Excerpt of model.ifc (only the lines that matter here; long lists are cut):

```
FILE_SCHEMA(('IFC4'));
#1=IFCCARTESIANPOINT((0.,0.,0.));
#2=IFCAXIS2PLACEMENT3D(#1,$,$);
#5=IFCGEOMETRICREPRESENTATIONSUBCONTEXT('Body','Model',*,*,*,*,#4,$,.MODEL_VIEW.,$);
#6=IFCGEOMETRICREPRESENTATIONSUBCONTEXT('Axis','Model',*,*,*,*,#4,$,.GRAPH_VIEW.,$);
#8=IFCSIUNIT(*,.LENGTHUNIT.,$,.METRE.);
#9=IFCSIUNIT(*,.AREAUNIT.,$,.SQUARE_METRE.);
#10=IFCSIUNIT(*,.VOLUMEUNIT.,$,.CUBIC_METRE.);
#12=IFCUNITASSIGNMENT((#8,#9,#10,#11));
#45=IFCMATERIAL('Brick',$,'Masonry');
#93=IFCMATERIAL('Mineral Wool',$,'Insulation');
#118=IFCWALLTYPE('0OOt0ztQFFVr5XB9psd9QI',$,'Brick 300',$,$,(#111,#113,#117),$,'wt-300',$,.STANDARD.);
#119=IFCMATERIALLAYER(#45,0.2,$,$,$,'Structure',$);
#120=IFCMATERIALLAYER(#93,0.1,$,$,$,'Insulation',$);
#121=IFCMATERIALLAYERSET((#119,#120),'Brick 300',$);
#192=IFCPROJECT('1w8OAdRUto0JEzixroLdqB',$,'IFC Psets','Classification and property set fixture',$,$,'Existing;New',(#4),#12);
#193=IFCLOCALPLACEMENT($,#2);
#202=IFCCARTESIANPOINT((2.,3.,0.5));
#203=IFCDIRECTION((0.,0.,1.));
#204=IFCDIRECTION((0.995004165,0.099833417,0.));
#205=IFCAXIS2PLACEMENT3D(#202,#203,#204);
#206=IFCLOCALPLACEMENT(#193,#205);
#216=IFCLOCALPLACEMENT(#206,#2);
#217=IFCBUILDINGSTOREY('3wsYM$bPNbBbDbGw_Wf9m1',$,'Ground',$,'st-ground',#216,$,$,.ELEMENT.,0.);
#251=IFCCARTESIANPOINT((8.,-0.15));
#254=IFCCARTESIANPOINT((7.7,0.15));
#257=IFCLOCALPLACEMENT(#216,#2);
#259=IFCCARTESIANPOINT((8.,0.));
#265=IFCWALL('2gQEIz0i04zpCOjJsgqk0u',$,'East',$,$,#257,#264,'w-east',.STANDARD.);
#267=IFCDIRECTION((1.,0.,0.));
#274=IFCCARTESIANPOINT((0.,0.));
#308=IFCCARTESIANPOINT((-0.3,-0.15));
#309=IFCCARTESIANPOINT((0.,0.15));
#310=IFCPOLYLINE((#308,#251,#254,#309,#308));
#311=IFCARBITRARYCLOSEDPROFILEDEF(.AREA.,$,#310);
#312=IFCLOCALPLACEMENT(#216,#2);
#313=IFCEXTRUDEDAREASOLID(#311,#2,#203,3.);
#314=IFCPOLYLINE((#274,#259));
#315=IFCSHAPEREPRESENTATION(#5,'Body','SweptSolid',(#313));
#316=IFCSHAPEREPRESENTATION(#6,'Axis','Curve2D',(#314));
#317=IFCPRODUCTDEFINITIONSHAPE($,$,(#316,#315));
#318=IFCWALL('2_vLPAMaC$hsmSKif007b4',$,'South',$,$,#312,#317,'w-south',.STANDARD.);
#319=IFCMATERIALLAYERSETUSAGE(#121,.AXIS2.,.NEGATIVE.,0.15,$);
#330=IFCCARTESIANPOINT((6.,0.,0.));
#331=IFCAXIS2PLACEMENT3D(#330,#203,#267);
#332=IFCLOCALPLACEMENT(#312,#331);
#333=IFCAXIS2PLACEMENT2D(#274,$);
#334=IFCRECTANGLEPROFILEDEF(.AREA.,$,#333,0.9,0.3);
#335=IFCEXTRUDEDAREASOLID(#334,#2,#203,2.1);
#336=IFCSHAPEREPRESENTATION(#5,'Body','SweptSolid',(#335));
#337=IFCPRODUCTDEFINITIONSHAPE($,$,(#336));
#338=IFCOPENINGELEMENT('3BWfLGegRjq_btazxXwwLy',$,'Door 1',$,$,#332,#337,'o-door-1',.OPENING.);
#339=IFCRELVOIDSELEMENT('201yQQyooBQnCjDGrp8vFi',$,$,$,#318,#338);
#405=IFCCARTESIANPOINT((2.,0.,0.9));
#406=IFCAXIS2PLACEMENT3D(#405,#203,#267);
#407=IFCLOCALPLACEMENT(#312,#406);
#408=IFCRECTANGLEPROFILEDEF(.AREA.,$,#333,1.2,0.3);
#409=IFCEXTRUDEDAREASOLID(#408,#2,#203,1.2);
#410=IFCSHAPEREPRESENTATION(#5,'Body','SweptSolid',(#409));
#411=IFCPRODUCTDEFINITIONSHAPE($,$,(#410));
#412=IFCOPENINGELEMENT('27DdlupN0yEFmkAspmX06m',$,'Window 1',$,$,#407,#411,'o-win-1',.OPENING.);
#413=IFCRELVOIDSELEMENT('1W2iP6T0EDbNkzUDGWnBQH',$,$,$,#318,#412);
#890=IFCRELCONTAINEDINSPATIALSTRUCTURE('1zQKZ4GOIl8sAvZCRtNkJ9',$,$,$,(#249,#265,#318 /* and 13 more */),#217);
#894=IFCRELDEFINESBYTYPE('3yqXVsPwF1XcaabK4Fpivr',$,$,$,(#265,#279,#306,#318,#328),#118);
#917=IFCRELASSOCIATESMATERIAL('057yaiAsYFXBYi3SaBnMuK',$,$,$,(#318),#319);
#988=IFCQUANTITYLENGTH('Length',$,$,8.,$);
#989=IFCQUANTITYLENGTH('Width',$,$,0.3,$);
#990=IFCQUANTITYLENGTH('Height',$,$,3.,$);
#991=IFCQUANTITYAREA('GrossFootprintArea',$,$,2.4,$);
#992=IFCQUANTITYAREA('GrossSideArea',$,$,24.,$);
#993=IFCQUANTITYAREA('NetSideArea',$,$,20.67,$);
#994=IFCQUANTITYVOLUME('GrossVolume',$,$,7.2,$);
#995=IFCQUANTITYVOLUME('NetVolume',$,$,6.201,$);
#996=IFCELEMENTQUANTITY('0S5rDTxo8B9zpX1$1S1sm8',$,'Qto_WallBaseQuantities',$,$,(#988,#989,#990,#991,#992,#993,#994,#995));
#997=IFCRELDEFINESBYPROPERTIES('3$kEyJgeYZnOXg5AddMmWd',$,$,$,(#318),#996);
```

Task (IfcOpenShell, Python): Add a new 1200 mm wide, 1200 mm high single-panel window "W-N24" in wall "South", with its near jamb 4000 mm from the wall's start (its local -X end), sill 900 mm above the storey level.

```python
import numpy as np
import ifcopenshell
import ifcopenshell.api.feature
import ifcopenshell.api.geometry
import ifcopenshell.api.pset
import ifcopenshell.api.root
import ifcopenshell.api.spatial
import ifcopenshell.geom
import ifcopenshell.util.element
import ifcopenshell.util.placement
import ifcopenshell.util.representation
import ifcopenshell.util.shape
import ifcopenshell.util.unit

model = ifcopenshell.open("model.ifc")
unit_scale = ifcopenshell.util.unit.calculate_unit_scale(model)
area_scale = ifcopenshell.util.unit.calculate_unit_scale(model, "AREAUNIT")
volume_scale = ifcopenshell.util.unit.calculate_unit_scale(model, "VOLUMEUNIT")
settings = ifcopenshell.geom.settings()


def volume(element):
    """Net volume in cubic metres, openings subtracted."""
    shape = ifcopenshell.geom.create_shape(settings, element)
    return ifcopenshell.util.shape.get_volume(shape.geometry)


wall = model.by_guid("2_vLPAMaC$hsmSKif007b4")
storey = ifcopenshell.util.element.get_container(wall, ifc_class="IfcBuildingStorey")
context = ifcopenshell.util.representation.get_context(model, "Model", "Body", "MODEL_VIEW")
before = volume(wall)

width, height, from_end, sill = 1.2, 1.2, 4, 0.9  # metres

# The wall runs along its own X axis, and the end named is its -X end.
wall_shape = ifcopenshell.geom.create_shape(settings, wall)
x, y, z = ifcopenshell.util.shape.get_vertices(wall_shape.geometry).T
start = x.min() + from_end
face, thickness = float(y.min()), float(y.max() - y.min())
wall_matrix = ifcopenshell.util.placement.get_local_placement(wall.ObjectPlacement)
level = ifcopenshell.util.placement.get_local_placement(storey.ObjectPlacement)[2, 3]


def in_wall(x, y):
    """Placement at x, y metres in the wall's axes, at sill height."""
    matrix = wall_matrix.copy()
    matrix[:, 3] = wall_matrix @ np.array([x / unit_scale, y / unit_scale, 0.0, 1.0])
    matrix[2, 3] = level + sill / unit_scale
    return matrix


# Opening: a box that overshoots both wall faces by 50 mm.
opening = ifcopenshell.api.root.create_entity(model, ifc_class="IfcOpeningElement", predefined_type="OPENING")
box = ifcopenshell.api.geometry.add_wall_representation(
    model, context=context, length=width, height=height, thickness=thickness + 0.1
)
ifcopenshell.api.geometry.assign_representation(model, product=opening, representation=box)
ifcopenshell.api.geometry.edit_object_placement(model, product=opening, matrix=in_wall(start, face - 0.05), is_si=False)
ifcopenshell.api.feature.add_feature(model, feature=opening, element=wall)

window = ifcopenshell.api.root.create_entity(model, ifc_class="IfcWindow", name="W-N24", predefined_type="WINDOW")
window.OverallWidth, window.OverallHeight = width / unit_scale, height / unit_scale
window.PartitioningType = "SINGLE_PANEL"
body = ifcopenshell.api.geometry.add_window_representation(
    model,
    context=context,
    overall_width=window.OverallWidth,
    overall_height=window.OverallHeight,
    partition_type="SINGLE_PANEL",
)
ifcopenshell.api.geometry.assign_representation(model, product=window, representation=body)
ifcopenshell.api.spatial.assign_container(model, products=[window], relating_structure=storey)
ifcopenshell.api.feature.add_filling(model, opening=opening, element=window)

# Centre the window in the wall's thickness.
ifcopenshell.api.geometry.edit_object_placement(model, product=window, matrix=in_wall(start, face), is_si=False)
window_shape = ifcopenshell.geom.create_shape(settings, window)
depth = ifcopenshell.util.shape.get_vertices(window_shape.geometry)[:, 1]
offset = face + thickness / 2 - (depth.min() + depth.max()) / 2
ifcopenshell.api.geometry.edit_object_placement(model, product=window, matrix=in_wall(start, offset), is_si=False)

after = volume(wall)

# Update the wall's stored quantities.
qto = model.by_id(ifcopenshell.util.element.get_pset(wall, "Qto_WallBaseQuantities", should_inherit=False)["id"])
ifcopenshell.api.pset.edit_qto(model, qto=qto, properties={
    "NetSideArea": after / thickness / area_scale,
    "NetVolume": after / volume_scale,
})

print(f"wall volume {before:.3f} -> {after:.3f} m3")

model.write("model_edited.ifc")
```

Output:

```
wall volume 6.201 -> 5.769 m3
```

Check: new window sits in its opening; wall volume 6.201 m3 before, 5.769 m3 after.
